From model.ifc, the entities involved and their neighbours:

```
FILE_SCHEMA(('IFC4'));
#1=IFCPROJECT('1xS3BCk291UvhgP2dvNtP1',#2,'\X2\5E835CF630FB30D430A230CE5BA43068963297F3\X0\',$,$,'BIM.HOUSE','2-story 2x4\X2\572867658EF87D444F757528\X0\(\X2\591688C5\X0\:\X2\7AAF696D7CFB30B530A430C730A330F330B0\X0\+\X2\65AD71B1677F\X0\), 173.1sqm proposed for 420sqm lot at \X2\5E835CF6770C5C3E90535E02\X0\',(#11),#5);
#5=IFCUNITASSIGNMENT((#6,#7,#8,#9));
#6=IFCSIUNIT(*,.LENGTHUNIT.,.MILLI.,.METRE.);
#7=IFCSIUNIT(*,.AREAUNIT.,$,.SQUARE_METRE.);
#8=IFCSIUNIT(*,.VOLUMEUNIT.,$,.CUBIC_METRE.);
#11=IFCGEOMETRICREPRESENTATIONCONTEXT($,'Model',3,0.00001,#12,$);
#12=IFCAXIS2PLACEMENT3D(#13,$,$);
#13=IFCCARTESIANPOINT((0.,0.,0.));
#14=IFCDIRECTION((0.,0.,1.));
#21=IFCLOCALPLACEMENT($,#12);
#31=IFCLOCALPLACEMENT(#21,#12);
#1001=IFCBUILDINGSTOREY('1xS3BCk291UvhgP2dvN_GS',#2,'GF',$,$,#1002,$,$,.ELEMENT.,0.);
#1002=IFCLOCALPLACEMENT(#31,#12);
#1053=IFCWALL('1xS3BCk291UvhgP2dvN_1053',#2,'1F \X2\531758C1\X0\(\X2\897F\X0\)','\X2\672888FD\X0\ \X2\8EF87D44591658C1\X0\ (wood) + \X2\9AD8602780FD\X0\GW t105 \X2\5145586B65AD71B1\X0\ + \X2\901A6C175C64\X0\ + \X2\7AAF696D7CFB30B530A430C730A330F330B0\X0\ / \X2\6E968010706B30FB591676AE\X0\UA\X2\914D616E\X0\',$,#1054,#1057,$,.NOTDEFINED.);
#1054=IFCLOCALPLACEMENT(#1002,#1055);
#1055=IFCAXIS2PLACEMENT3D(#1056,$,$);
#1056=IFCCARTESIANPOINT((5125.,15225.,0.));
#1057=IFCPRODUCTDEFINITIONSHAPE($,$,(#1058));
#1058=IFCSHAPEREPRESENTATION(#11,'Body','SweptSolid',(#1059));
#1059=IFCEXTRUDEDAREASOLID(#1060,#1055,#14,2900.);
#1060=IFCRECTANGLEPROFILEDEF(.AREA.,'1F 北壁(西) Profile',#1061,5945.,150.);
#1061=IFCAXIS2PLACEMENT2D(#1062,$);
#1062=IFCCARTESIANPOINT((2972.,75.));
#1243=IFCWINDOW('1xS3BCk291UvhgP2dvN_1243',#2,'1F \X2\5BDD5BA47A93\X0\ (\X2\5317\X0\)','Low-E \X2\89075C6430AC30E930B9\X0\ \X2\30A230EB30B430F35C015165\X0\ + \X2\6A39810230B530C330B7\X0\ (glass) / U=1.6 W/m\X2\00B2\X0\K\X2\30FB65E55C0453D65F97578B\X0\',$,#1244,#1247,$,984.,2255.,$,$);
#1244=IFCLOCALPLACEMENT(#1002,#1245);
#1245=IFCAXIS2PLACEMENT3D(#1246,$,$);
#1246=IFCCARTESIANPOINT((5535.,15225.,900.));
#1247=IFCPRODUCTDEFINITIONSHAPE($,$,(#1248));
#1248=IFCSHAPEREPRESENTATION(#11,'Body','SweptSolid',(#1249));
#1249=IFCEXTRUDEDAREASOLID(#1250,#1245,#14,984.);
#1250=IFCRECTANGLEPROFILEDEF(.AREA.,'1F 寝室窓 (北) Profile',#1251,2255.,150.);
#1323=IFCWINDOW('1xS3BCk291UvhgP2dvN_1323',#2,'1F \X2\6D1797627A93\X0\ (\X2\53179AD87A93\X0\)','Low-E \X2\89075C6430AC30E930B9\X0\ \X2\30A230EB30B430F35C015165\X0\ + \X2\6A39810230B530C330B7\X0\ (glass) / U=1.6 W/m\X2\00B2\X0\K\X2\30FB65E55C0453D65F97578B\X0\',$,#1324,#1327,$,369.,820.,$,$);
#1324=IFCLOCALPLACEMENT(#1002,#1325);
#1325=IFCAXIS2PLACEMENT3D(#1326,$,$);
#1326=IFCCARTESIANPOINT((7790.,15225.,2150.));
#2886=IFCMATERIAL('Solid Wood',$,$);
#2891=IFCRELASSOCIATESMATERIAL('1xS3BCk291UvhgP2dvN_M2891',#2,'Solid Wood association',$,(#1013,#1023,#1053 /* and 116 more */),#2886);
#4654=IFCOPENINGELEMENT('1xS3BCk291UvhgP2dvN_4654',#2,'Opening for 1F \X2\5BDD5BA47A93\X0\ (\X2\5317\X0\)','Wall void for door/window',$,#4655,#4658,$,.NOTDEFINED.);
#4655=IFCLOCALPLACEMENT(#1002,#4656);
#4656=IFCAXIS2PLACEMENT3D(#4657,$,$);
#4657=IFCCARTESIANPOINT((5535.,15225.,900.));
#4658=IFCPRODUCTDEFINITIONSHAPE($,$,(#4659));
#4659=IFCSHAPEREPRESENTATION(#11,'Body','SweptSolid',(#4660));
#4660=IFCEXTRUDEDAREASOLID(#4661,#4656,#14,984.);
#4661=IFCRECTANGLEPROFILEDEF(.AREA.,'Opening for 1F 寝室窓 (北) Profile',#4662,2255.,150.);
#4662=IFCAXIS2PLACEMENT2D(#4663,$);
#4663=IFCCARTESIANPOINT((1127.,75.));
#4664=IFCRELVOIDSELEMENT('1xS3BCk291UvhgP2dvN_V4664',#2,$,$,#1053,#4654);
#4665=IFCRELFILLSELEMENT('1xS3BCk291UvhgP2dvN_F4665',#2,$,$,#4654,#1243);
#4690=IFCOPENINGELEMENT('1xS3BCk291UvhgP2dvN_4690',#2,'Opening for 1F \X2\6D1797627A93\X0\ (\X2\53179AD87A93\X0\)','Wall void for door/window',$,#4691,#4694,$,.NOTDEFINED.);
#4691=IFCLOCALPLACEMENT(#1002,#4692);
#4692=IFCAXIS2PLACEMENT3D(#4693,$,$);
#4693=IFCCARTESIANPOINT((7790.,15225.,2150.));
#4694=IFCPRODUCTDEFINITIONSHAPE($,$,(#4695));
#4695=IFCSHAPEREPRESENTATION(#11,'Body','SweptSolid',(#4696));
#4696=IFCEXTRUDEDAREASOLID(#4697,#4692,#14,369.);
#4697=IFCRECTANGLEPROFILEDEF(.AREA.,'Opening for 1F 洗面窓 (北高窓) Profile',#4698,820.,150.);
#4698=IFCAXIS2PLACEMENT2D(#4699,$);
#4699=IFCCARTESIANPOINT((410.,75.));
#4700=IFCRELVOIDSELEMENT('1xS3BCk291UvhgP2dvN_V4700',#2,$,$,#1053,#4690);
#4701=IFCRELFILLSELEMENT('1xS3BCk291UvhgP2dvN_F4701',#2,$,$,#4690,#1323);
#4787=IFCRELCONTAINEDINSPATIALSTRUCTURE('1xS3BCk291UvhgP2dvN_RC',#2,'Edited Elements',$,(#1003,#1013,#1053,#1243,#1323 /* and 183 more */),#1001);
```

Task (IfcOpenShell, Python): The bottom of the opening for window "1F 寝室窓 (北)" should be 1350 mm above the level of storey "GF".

```python
import numpy as np
import ifcopenshell
import ifcopenshell.api.geometry
import ifcopenshell.geom
import ifcopenshell.util.element
import ifcopenshell.util.placement
import ifcopenshell.util.shape
import ifcopenshell.util.unit

model = ifcopenshell.open("model.ifc")
unit_scale = ifcopenshell.util.unit.calculate_unit_scale(model)

window = model.by_guid("1xS3BCk291UvhgP2dvN_1243")
opening = window.FillsVoids[0].RelatingOpeningElement
storey = ifcopenshell.util.element.get_container(window, ifc_class="IfcBuildingStorey")
level = ifcopenshell.util.placement.get_local_placement(storey.ObjectPlacement)[2, 3]

# The opening's origin need not be at the sill, so measure its lowest point.
shape = ifcopenshell.geom.create_shape(ifcopenshell.geom.settings(), opening)
bottom = ifcopenshell.util.shape.get_shape_bottom_elevation(shape, shape.geometry) / unit_scale
dz = level + 1350.0 - bottom

shift = np.array([0.0, 0.0, dz])
# The window is not placed relative to its opening, so move both.
for product in (opening, window):
    matrix = ifcopenshell.util.placement.get_local_placement(product.ObjectPlacement)
    matrix[:3, 3] += shift
    ifcopenshell.api.geometry.edit_object_placement(model, product=product, matrix=matrix, is_si=False)

print(f"moved by {dz * unit_scale:+.3f} m")

model.write("model_rev.ifc")
```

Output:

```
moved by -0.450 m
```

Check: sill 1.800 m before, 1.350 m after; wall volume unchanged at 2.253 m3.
